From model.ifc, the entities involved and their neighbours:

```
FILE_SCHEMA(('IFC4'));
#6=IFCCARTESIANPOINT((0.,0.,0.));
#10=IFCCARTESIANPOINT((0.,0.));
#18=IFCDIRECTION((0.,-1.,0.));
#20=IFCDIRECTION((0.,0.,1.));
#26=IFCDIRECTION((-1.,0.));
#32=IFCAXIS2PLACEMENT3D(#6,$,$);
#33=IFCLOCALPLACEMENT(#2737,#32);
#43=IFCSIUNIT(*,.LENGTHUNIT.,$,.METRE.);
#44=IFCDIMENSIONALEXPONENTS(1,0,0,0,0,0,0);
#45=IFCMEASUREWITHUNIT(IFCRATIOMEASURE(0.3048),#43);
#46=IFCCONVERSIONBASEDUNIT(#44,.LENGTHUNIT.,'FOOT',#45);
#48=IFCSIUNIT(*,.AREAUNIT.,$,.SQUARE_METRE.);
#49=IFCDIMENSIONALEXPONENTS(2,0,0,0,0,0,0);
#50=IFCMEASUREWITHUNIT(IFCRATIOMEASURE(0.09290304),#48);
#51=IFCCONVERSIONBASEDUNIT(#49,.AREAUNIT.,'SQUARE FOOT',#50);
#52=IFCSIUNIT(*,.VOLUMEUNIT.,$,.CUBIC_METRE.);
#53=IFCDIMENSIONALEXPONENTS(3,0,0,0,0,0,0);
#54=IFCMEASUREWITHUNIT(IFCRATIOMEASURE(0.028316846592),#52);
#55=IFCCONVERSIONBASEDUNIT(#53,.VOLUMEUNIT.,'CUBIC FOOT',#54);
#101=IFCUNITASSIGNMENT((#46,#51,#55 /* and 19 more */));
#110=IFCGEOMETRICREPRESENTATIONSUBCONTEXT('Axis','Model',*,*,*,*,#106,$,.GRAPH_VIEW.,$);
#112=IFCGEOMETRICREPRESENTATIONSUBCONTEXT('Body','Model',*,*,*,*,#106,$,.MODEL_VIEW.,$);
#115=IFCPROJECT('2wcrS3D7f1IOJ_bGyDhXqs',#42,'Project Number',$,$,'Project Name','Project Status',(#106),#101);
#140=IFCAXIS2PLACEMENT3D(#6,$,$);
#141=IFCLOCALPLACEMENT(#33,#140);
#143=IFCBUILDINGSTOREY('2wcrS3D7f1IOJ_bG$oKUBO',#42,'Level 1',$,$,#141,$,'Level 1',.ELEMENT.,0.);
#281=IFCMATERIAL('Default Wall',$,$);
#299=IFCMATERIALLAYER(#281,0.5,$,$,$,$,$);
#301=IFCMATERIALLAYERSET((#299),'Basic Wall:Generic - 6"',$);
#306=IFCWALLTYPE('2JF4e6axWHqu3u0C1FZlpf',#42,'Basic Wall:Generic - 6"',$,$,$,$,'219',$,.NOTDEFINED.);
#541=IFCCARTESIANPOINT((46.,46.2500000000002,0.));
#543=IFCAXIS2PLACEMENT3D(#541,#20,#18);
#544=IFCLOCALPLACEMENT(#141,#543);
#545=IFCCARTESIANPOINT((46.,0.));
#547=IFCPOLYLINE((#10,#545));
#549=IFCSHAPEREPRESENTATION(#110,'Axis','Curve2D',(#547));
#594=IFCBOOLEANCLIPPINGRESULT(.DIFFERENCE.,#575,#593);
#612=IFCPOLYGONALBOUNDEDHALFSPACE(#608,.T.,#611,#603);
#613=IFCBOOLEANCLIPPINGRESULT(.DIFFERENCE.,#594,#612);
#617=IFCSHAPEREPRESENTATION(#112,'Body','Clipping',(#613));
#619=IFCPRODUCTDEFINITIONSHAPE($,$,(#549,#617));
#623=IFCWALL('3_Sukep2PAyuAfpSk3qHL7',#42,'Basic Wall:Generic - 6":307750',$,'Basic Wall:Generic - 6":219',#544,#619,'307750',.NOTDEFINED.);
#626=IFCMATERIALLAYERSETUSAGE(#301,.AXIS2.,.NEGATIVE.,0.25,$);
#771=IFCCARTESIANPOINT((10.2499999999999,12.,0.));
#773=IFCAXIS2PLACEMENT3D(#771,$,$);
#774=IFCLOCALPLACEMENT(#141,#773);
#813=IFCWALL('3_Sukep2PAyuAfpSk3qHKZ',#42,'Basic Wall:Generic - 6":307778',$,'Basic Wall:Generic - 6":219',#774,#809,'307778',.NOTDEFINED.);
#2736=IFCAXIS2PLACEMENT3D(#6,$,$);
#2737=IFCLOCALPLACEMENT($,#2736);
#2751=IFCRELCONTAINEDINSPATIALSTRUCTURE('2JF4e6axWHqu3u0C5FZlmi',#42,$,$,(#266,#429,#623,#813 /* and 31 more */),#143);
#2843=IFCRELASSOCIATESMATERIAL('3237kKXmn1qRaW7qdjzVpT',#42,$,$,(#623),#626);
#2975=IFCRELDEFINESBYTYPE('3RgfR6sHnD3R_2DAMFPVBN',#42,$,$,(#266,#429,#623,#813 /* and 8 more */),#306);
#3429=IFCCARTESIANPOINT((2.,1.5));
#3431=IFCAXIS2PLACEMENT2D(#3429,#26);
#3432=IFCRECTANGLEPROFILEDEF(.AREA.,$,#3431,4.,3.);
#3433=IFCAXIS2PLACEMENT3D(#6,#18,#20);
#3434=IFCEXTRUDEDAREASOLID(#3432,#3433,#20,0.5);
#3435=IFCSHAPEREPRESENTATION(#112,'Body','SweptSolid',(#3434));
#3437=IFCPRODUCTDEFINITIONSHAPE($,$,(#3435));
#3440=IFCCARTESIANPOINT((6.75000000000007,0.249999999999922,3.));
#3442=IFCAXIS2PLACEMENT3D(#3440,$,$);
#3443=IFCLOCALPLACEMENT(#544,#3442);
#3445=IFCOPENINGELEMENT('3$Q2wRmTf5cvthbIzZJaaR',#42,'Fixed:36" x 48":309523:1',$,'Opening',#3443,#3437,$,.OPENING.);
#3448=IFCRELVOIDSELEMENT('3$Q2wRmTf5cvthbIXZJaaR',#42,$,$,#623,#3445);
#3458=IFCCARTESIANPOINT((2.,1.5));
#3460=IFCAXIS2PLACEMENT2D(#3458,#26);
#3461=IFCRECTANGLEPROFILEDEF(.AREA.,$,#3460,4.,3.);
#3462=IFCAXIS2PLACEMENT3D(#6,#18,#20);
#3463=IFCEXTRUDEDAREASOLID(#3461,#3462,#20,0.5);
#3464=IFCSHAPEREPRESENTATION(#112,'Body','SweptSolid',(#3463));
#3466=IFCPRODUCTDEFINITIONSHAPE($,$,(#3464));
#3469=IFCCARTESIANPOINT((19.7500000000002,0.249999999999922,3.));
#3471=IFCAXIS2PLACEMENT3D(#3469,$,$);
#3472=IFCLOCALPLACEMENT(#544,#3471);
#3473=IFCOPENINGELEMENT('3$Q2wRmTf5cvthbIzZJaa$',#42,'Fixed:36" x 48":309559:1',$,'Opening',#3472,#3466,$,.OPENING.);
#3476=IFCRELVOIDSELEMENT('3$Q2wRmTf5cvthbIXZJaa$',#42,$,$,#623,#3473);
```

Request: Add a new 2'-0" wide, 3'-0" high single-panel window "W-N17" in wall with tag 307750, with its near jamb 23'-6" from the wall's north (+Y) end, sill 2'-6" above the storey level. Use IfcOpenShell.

```python
import numpy as np
import ifcopenshell
import ifcopenshell.api.feature
import ifcopenshell.api.geometry
import ifcopenshell.api.root
import ifcopenshell.api.spatial
import ifcopenshell.geom
import ifcopenshell.util.element
import ifcopenshell.util.placement
import ifcopenshell.util.representation
import ifcopenshell.util.shape
import ifcopenshell.util.unit

model = ifcopenshell.open("model.ifc")
unit_scale = ifcopenshell.util.unit.calculate_unit_scale(model)
settings = ifcopenshell.geom.settings()


def volume(element):
    """Net volume in cubic metres, openings subtracted."""
    shape = ifcopenshell.geom.create_shape(settings, element)
    return ifcopenshell.util.shape.get_volume(shape.geometry)


wall = model.by_guid("3_Sukep2PAyuAfpSk3qHL7")
storey = ifcopenshell.util.element.get_container(wall, ifc_class="IfcBuildingStorey")
context = ifcopenshell.util.representation.get_context(model, "Model", "Body", "MODEL_VIEW")
before = volume(wall)

width, height, from_end, sill = 0.6096, 0.9144, 7.1628, 0.762  # metres

# The wall runs along its own X axis, and the end named is its -X end.
wall_shape = ifcopenshell.geom.create_shape(settings, wall)
x, y, z = ifcopenshell.util.shape.get_vertices(wall_shape.geometry).T
start = x.min() + from_end
face, thickness = float(y.min()), float(y.max() - y.min())
wall_matrix = ifcopenshell.util.placement.get_local_placement(wall.ObjectPlacement)
level = ifcopenshell.util.placement.get_local_placement(storey.ObjectPlacement)[2, 3]


def in_wall(x, y):
    """Placement at x, y metres in the wall's axes, at sill height."""
    matrix = wall_matrix.copy()
    matrix[:, 3] = wall_matrix @ np.array([x / unit_scale, y / unit_scale, 0.0, 1.0])
    matrix[2, 3] = level + sill / unit_scale
    return matrix


# Opening: a box that overshoots both wall faces by 50 mm.
opening = ifcopenshell.api.root.create_entity(model, ifc_class="IfcOpeningElement", predefined_type="OPENING")
box = ifcopenshell.api.geometry.add_wall_representation(
    model, context=context, length=width, height=height, thickness=thickness + 0.1
)
ifcopenshell.api.geometry.assign_representation(model, product=opening, representation=box)
ifcopenshell.api.geometry.edit_object_placement(model, product=opening, matrix=in_wall(start, face - 0.05), is_si=False)
ifcopenshell.api.feature.add_feature(model, feature=opening, element=wall)

window = ifcopenshell.api.root.create_entity(model, ifc_class="IfcWindow", name="W-N17", predefined_type="WINDOW")
window.OverallWidth, window.OverallHeight = width / unit_scale, height / unit_scale
window.PartitioningType = "SINGLE_PANEL"
body = ifcopenshell.api.geometry.add_window_representation(
    model,
    context=context,
    overall_width=window.OverallWidth,
    overall_height=window.OverallHeight,
    partition_type="SINGLE_PANEL",
)
ifcopenshell.api.geometry.assign_representation(model, product=window, representation=body)
ifcopenshell.api.spatial.assign_container(model, products=[window], relating_structure=storey)
ifcopenshell.api.feature.add_filling(model, opening=opening, element=window)

# Centre the window in the wall's thickness.
ifcopenshell.api.geometry.edit_object_placement(model, product=window, matrix=in_wall(start, face), is_si=False)
window_shape = ifcopenshell.geom.create_shape(settings, window)
depth = ifcopenshell.util.shape.get_vertices(window_shape.geometry)[:, 1]
offset = face + thickness / 2 - (depth.min() + depth.max()) / 2
ifcopenshell.api.geometry.edit_object_placement(model, product=window, matrix=in_wall(start, offset), is_si=False)

after = volume(wall)

print(f"wall volume {before:.3f} -> {after:.3f} m3")

model.write("model-out.ifc")
```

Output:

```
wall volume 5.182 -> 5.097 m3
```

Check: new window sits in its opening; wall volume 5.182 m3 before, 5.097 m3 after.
